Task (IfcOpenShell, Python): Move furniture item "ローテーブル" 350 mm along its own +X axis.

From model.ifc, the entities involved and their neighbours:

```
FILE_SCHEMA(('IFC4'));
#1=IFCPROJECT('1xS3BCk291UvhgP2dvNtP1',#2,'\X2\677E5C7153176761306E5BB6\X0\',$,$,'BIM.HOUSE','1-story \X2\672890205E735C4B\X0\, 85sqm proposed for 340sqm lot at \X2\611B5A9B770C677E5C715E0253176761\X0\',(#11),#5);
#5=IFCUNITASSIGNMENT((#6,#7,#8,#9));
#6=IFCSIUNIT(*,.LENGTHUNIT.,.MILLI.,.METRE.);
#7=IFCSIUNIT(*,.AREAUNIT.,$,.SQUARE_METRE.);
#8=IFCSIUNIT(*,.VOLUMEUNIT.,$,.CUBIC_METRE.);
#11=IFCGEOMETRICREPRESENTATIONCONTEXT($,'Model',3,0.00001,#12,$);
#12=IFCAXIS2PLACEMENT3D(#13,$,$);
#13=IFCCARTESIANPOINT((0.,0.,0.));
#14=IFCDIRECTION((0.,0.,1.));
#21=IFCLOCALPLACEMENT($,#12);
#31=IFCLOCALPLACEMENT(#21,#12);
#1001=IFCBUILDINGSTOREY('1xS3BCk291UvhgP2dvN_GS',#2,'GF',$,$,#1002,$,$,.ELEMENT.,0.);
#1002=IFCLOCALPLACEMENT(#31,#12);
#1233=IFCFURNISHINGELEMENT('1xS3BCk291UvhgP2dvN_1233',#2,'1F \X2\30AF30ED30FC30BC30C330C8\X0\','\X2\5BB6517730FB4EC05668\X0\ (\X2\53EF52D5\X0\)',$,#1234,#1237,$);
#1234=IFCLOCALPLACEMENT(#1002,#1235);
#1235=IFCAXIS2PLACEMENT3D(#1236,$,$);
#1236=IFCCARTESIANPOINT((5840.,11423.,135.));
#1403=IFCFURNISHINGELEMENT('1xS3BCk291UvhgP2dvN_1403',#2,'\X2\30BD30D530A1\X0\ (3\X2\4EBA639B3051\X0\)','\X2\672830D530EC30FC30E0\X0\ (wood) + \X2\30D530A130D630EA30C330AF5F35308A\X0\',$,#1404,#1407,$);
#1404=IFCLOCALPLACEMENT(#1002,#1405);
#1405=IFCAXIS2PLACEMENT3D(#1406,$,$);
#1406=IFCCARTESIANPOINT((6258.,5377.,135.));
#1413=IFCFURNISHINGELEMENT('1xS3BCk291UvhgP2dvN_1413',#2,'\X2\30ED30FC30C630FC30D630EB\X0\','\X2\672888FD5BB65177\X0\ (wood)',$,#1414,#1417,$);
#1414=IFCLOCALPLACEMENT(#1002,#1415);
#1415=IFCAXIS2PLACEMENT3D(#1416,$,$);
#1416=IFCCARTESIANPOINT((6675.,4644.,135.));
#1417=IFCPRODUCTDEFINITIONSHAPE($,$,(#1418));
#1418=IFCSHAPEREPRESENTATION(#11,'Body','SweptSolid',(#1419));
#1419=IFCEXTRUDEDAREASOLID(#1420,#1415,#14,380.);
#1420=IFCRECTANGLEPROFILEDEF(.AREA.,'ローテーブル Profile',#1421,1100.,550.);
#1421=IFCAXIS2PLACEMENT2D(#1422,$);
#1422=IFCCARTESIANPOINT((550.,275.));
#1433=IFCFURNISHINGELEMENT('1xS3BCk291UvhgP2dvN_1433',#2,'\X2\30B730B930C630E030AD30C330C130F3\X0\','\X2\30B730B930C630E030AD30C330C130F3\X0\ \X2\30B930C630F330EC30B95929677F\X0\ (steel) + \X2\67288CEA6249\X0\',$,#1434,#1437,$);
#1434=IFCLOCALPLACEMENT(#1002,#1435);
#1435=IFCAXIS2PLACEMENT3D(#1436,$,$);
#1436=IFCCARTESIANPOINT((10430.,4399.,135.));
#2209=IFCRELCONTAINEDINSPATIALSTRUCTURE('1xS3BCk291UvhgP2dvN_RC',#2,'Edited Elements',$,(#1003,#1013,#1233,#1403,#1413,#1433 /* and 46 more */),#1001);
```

```python
import ifcopenshell
import ifcopenshell.api.geometry
import ifcopenshell.util.placement
import ifcopenshell.util.unit

model = ifcopenshell.open("model.ifc")
unit_scale = ifcopenshell.util.unit.calculate_unit_scale(model)

item = model.by_id(1413)
matrix = ifcopenshell.util.placement.get_local_placement(item.ObjectPlacement)
matrix[:3, 3] += matrix[:3, 0] * 0.35 / unit_scale
ifcopenshell.api.geometry.edit_object_placement(model, product=item, matrix=matrix, is_si=False)

print(ifcopenshell.util.placement.get_local_placement(item.ObjectPlacement).round(3) + 0.0)

model.write("model-out.ifc")
```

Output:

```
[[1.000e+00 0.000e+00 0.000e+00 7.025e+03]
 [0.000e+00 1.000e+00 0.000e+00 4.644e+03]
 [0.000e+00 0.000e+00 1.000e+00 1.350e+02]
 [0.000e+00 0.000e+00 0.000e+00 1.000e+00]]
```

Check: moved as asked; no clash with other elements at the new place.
